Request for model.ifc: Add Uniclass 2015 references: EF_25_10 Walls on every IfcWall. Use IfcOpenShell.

First a look at what the model holds.

```python
import ifcopenshell

model = ifcopenshell.open("model.ifc")
print(model.schema)
print("classifications:", [c.Name for c in model.by_type("IfcClassification")])
for ifc_class in ("IfcDoor", "IfcRoof", "IfcStair", "IfcWall", "IfcWindow"):
    print(ifc_class, len(model.by_type(ifc_class)))
```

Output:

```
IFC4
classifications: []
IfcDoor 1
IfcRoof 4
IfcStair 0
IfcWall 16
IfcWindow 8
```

```python
import ifcopenshell
import ifcopenshell.api.classification

model = ifcopenshell.open("model.ifc")

system = ifcopenshell.api.classification.add_classification(model, classification="Uniclass 2015")

codes = {
    "IfcWall": ("EF_25_10", "Walls"),
}
for ifc_class, (code, name) in codes.items():
    products = model.by_type(ifc_class)
    ifcopenshell.api.classification.add_reference(
        model, products=products, classification=system, identification=code, name=name
    )
    print(code, len(products))

model.write("model_v2.ifc")
```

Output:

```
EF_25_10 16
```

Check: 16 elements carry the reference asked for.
